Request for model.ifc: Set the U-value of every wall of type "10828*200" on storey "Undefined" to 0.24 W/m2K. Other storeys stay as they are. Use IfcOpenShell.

First a look at what the model holds.

```python
import ifcopenshell
import ifcopenshell.util.element

model = ifcopenshell.open("model.ifc")
print(model.schema)
storey = next(s for s in model.by_type("IfcBuildingStorey") if s.Name == "Undefined")
walls = [e for e in ifcopenshell.util.element.get_decomposition(storey) if e.is_a("IfcWall")]
seen = {}
for e in walls:
    element_type = ifcopenshell.util.element.get_type(e)
    key = (element_type.Name if element_type != e and element_type else None, ifcopenshell.util.element.get_pset(e, "Pset_WallCommon", "ThermalTransmittance"))
    seen[key] = seen.get(key, 0) + 1
for (name, value), count in sorted(seen.items(), key=str):
    print(count, "x", name, "|", value)
```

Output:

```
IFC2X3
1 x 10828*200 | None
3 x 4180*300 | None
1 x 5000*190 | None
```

```python
import ifcopenshell
import ifcopenshell.api.pset
import ifcopenshell.util.element

model = ifcopenshell.open("model.ifc")

storey = next(s for s in model.by_type("IfcBuildingStorey") if s.Name == "Undefined")
walls = [e for e in ifcopenshell.util.element.get_decomposition(storey) if e.is_a("IfcWall")]

count = 0
for e in walls:
    element_type = ifcopenshell.util.element.get_type(e)
    if element_type in (None, e) or element_type.Name != "10828*200":
        continue
    # add_pset returns the element's existing set when there is one.
    pset = ifcopenshell.api.pset.add_pset(model, product=e, name="Pset_WallCommon")
    ifcopenshell.api.pset.edit_pset(model, pset=pset, properties={"ThermalTransmittance": 0.24})
    count += 1

print(count, "walls updated")

model.write("model_v2.ifc")
```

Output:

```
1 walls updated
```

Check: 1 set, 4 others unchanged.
